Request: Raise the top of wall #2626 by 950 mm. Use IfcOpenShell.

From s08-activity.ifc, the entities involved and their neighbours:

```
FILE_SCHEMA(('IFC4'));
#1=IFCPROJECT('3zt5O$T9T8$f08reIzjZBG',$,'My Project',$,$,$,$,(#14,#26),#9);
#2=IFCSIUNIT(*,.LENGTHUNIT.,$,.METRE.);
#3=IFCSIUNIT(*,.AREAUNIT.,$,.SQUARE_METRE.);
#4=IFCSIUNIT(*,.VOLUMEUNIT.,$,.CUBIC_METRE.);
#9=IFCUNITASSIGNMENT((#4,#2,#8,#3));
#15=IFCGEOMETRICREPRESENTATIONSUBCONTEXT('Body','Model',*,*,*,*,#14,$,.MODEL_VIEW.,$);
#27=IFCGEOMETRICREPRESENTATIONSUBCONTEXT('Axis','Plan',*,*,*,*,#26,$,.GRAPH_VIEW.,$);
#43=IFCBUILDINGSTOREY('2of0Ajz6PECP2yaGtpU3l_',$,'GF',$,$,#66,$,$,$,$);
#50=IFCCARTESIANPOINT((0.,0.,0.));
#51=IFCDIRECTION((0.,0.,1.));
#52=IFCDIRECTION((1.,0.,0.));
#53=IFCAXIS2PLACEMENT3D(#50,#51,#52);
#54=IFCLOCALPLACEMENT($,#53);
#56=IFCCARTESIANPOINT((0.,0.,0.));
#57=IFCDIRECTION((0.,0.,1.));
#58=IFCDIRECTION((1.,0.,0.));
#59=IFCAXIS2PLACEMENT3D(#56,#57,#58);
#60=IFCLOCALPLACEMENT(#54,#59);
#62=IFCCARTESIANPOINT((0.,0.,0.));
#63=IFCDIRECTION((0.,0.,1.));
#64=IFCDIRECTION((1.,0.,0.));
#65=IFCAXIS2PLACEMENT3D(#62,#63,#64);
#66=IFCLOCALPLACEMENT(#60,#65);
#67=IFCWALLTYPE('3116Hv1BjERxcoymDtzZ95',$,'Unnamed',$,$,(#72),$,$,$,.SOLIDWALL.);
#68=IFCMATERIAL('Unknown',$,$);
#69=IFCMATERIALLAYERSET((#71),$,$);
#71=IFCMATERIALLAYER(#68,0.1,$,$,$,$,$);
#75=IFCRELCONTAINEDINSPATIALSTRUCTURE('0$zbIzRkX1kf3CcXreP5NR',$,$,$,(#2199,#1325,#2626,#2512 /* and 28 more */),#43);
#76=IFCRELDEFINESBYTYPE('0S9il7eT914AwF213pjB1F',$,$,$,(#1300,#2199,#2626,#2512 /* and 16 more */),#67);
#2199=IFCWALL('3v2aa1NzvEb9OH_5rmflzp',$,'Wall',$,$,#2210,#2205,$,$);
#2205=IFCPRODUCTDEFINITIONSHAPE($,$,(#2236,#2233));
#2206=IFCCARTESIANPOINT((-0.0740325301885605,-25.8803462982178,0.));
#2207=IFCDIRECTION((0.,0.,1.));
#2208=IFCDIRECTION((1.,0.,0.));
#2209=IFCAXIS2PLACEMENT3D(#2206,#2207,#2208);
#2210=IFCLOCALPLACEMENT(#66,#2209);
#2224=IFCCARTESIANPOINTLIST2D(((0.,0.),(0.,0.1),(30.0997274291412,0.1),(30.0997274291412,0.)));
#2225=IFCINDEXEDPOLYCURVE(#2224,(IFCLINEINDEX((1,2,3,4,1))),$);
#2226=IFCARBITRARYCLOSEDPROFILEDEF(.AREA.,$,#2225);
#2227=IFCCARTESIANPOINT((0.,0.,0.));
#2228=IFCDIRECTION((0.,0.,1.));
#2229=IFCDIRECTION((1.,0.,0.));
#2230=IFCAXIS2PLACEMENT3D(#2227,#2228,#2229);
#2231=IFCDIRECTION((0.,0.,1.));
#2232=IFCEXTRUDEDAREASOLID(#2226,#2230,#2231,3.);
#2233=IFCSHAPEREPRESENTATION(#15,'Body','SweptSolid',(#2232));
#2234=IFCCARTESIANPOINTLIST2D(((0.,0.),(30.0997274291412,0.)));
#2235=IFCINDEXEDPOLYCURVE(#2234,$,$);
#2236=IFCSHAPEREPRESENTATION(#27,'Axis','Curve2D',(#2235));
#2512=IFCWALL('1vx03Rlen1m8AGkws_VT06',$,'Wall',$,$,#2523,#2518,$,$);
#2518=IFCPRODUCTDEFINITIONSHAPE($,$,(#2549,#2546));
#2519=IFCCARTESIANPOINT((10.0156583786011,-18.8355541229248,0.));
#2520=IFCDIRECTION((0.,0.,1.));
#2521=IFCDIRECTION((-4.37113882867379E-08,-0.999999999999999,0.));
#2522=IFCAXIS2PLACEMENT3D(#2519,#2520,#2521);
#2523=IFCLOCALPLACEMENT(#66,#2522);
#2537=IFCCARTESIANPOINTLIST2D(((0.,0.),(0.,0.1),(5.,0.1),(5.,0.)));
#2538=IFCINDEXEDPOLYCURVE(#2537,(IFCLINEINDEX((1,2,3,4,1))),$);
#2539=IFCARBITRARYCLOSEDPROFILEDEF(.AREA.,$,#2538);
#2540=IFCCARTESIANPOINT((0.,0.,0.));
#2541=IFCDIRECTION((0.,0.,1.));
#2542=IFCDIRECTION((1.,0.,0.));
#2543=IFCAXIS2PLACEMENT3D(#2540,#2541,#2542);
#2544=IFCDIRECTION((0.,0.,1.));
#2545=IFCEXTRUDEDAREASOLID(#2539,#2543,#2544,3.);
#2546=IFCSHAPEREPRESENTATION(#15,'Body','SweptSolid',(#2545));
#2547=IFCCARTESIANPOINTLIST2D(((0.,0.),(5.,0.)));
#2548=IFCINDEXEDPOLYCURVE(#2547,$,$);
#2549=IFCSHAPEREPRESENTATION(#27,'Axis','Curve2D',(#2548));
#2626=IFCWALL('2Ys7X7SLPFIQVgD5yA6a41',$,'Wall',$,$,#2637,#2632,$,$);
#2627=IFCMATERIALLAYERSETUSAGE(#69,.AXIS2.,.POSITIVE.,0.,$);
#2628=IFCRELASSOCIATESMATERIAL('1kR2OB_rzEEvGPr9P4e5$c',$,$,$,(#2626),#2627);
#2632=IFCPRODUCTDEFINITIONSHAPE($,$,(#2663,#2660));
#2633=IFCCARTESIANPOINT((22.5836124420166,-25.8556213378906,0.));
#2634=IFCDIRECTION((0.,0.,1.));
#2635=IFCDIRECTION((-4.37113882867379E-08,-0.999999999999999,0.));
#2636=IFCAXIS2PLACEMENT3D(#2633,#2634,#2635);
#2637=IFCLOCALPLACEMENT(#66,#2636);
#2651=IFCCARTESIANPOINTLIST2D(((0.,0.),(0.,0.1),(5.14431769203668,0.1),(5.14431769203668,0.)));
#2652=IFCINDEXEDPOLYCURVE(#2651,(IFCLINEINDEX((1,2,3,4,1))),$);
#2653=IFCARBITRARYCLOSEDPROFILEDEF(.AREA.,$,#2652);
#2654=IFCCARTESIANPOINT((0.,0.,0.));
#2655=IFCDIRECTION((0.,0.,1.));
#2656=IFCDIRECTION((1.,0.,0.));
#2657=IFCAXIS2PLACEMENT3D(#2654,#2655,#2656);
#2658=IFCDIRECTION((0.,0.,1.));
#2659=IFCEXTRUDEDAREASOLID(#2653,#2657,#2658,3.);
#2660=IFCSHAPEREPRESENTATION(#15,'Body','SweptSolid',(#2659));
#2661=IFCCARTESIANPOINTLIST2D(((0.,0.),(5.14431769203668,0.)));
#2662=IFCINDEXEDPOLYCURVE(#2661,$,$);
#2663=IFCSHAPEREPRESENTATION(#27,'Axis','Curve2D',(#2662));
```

```python
import ifcopenshell
import ifcopenshell.geom
import ifcopenshell.util.representation
import ifcopenshell.util.shape
import ifcopenshell.util.unit

model = ifcopenshell.open("s08-activity.ifc")
unit_scale = ifcopenshell.util.unit.calculate_unit_scale(model)
settings = ifcopenshell.geom.settings()


def volume(element):
    """Net volume in cubic metres, openings subtracted."""
    shape = ifcopenshell.geom.create_shape(settings, element)
    return ifcopenshell.util.shape.get_volume(shape.geometry)


wall = model.by_id(2626)
before = volume(wall)

body = ifcopenshell.util.representation.get_representation(wall, "Model", "Body")
solid = body.Items[0]
old_height = solid.Depth
solid.Depth += 0.95 / unit_scale
after = volume(wall)

print(f"height {old_height:g} -> {solid.Depth:g}, volume {before:.3f} -> {after:.3f} m3")

model.write("s08-activity_edited.ifc")
```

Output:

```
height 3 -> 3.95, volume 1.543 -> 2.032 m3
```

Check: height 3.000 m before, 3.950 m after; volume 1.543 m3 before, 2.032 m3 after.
